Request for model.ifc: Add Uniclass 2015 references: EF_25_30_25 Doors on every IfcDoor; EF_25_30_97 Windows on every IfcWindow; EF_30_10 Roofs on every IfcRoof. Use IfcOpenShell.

First a look at what the model holds.

```python
import ifcopenshell

model = ifcopenshell.open("model.ifc")
print(model.schema)
print("classifications:", [c.Name for c in model.by_type("IfcClassification")])
for ifc_class in ("IfcDoor", "IfcRoof", "IfcStair", "IfcWall", "IfcWindow"):
    print(ifc_class, len(model.by_type(ifc_class)))
```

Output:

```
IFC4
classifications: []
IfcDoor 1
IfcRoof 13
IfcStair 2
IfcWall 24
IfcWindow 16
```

```python
import ifcopenshell
import ifcopenshell.api.classification

model = ifcopenshell.open("model.ifc")

system = ifcopenshell.api.classification.add_classification(model, classification="Uniclass 2015")

codes = {
    "IfcDoor": ("EF_25_30_25", "Doors"),
    "IfcWindow": ("EF_25_30_97", "Windows"),
    "IfcRoof": ("EF_30_10", "Roofs"),
}
for ifc_class, (code, name) in codes.items():
    products = model.by_type(ifc_class)
    ifcopenshell.api.classification.add_reference(
        model, products=products, classification=system, identification=code, name=name
    )
    print(code, len(products))

model.write("model-out.ifc")
```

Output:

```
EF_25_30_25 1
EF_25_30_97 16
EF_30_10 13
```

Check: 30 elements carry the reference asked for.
